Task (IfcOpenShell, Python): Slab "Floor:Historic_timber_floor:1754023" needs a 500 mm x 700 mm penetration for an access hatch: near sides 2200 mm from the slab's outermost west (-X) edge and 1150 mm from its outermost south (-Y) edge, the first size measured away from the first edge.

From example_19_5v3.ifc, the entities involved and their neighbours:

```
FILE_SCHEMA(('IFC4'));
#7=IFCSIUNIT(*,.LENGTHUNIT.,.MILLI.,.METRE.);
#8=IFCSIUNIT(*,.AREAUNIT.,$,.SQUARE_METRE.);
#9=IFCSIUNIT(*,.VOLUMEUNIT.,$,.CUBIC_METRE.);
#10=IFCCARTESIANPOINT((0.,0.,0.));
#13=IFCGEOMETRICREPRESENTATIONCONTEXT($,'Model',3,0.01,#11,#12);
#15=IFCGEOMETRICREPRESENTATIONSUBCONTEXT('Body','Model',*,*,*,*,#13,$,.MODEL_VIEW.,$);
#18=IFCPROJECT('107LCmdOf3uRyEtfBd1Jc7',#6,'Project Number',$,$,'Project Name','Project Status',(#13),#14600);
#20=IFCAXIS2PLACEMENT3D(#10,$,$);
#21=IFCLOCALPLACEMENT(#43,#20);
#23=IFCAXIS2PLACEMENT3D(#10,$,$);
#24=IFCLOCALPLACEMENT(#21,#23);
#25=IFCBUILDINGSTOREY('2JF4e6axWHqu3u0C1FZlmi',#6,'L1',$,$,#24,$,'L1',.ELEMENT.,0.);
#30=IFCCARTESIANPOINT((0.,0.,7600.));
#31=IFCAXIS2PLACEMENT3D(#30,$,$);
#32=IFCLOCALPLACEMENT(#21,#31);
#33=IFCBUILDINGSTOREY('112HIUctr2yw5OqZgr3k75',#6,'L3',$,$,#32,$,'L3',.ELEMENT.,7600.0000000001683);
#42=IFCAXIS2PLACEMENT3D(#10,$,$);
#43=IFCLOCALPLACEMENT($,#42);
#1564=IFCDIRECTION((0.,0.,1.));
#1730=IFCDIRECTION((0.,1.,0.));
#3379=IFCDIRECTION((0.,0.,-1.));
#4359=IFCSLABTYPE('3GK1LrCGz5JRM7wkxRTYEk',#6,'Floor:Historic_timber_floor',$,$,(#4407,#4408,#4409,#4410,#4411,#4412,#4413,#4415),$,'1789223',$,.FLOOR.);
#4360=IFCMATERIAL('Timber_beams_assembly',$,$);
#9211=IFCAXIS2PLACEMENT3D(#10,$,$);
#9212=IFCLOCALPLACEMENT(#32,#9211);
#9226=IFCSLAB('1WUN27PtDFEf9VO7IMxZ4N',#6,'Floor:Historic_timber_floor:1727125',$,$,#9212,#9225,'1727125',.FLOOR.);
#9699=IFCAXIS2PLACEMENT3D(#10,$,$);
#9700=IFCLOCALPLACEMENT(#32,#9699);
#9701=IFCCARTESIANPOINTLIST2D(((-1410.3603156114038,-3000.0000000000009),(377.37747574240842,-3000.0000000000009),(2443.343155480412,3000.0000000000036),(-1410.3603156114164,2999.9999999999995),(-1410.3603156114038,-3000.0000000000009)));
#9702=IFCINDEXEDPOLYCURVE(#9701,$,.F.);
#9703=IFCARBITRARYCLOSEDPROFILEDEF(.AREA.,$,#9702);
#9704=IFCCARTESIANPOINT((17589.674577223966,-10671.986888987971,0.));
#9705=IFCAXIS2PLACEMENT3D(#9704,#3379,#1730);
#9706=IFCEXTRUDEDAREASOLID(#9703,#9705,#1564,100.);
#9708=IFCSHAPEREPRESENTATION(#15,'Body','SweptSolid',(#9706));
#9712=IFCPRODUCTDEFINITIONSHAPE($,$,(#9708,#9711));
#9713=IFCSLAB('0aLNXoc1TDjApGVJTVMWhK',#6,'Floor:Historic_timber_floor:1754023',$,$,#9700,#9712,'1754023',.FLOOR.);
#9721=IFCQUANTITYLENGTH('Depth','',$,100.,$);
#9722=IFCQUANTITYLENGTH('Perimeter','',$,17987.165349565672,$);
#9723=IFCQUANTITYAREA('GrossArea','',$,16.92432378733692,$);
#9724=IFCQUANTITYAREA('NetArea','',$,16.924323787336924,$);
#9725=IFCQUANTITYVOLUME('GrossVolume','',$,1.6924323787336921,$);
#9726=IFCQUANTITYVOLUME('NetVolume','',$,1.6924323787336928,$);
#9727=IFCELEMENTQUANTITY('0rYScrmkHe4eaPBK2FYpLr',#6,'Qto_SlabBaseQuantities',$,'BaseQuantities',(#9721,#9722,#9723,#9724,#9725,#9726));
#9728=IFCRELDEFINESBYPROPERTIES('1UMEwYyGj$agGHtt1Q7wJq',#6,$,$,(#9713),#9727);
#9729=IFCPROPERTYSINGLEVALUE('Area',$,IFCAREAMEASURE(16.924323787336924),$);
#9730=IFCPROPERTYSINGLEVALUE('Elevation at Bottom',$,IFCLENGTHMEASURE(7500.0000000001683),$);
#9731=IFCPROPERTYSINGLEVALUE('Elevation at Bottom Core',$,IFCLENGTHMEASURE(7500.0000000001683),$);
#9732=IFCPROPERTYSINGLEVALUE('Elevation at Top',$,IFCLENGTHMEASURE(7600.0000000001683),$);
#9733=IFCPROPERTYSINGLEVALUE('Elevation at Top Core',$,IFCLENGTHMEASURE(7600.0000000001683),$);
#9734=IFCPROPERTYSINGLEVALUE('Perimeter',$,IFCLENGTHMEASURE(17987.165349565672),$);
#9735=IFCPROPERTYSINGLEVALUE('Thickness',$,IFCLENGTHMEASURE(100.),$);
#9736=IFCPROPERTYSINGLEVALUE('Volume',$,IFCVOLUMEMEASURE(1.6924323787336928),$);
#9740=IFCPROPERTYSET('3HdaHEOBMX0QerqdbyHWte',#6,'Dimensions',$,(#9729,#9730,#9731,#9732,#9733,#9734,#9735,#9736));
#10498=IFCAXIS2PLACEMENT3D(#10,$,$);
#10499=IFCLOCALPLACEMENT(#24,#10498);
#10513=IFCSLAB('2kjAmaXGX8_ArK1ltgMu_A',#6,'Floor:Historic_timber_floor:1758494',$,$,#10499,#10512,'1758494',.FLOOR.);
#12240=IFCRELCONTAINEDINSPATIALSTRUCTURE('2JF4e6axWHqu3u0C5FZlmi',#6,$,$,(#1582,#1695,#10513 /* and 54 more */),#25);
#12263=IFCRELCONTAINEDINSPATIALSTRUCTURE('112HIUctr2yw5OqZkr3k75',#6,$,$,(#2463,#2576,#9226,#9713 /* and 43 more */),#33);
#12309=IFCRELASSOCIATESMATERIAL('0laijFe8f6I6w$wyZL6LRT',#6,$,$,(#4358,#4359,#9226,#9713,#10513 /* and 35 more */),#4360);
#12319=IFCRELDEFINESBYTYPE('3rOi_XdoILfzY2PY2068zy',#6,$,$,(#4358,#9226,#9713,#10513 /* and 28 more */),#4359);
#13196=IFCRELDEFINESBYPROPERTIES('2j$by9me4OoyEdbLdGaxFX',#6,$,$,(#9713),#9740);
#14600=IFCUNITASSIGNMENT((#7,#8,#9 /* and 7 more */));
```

```python
import numpy as np
import ifcopenshell
import ifcopenshell.api.feature
import ifcopenshell.api.geometry
import ifcopenshell.api.pset
import ifcopenshell.api.root
import ifcopenshell.geom
import ifcopenshell.util.element
import ifcopenshell.util.placement
import ifcopenshell.util.representation
import ifcopenshell.util.shape
import ifcopenshell.util.unit

model = ifcopenshell.open("example_19_5v3.ifc")
unit_scale = ifcopenshell.util.unit.calculate_unit_scale(model)
area_scale = ifcopenshell.util.unit.calculate_unit_scale(model, "AREAUNIT")
volume_scale = ifcopenshell.util.unit.calculate_unit_scale(model, "VOLUMEUNIT")
settings = ifcopenshell.geom.settings()


def volume(element):
    """Net volume in cubic metres, openings subtracted."""
    shape = ifcopenshell.geom.create_shape(settings, element)
    return ifcopenshell.util.shape.get_volume(shape.geometry)


slab = model.by_guid("0aLNXoc1TDjApGVJTVMWhK")
before = volume(slab)

# Extent in the slab's own axes, in metres. The edges named are its -X and -Y sides.
slab_shape = ifcopenshell.geom.create_shape(settings, slab)
vertices = ifcopenshell.util.shape.get_vertices(slab_shape.geometry)
x_min, y_min, bottom = vertices.min(axis=0)
top = vertices[:, 2].max()

opening = ifcopenshell.api.root.create_entity(model, ifc_class="IfcOpeningElement", name="Access hatch opening", predefined_type="OPENING")
context = ifcopenshell.util.representation.get_context(model, "Model", "Body", "MODEL_VIEW")
width, depth = 0.5, 0.7
outline = [(0.0, 0.0), (width, 0.0), (width, depth), (0.0, depth), (0.0, 0.0)]
# Overshoot both faces by 50 mm so the cut is clean.
shape = ifcopenshell.api.geometry.add_slab_representation(
    model, context=context, depth=top - bottom + 0.1, polyline=outline
)
ifcopenshell.api.geometry.assign_representation(model, product=opening, representation=shape)

matrix = ifcopenshell.util.placement.get_local_placement(slab.ObjectPlacement)
matrix[:, 3] = matrix @ np.append(np.array([x_min + 2.2, y_min + 1.15, bottom - 0.05]) / unit_scale, 1.0)
ifcopenshell.api.geometry.edit_object_placement(model, product=opening, matrix=matrix, is_si=False)
ifcopenshell.api.feature.add_feature(model, feature=opening, element=slab)

after = volume(slab)

# Update the slab's stored quantities.
qto = model.by_id(ifcopenshell.util.element.get_pset(slab, "Qto_SlabBaseQuantities", should_inherit=False)["id"])
ifcopenshell.api.pset.edit_qto(model, qto=qto, properties={
    "NetArea": after / (top - bottom) / area_scale,
    "NetVolume": after / volume_scale,
})
pset = model.by_id(ifcopenshell.util.element.get_pset(slab, "Dimensions", should_inherit=False)["id"])
ifcopenshell.api.pset.edit_pset(model, pset=pset, properties={
    "Area": model.create_entity("IfcAreaMeasure", after / (top - bottom) / area_scale),
    "Volume": model.create_entity("IfcVolumeMeasure", after / volume_scale),
})

print(f"slab volume {before:.3f} -> {after:.3f} m3")

model.write("example_19_5v3_v2.ifc")
```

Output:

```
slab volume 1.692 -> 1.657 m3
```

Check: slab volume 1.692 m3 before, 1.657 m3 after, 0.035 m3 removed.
